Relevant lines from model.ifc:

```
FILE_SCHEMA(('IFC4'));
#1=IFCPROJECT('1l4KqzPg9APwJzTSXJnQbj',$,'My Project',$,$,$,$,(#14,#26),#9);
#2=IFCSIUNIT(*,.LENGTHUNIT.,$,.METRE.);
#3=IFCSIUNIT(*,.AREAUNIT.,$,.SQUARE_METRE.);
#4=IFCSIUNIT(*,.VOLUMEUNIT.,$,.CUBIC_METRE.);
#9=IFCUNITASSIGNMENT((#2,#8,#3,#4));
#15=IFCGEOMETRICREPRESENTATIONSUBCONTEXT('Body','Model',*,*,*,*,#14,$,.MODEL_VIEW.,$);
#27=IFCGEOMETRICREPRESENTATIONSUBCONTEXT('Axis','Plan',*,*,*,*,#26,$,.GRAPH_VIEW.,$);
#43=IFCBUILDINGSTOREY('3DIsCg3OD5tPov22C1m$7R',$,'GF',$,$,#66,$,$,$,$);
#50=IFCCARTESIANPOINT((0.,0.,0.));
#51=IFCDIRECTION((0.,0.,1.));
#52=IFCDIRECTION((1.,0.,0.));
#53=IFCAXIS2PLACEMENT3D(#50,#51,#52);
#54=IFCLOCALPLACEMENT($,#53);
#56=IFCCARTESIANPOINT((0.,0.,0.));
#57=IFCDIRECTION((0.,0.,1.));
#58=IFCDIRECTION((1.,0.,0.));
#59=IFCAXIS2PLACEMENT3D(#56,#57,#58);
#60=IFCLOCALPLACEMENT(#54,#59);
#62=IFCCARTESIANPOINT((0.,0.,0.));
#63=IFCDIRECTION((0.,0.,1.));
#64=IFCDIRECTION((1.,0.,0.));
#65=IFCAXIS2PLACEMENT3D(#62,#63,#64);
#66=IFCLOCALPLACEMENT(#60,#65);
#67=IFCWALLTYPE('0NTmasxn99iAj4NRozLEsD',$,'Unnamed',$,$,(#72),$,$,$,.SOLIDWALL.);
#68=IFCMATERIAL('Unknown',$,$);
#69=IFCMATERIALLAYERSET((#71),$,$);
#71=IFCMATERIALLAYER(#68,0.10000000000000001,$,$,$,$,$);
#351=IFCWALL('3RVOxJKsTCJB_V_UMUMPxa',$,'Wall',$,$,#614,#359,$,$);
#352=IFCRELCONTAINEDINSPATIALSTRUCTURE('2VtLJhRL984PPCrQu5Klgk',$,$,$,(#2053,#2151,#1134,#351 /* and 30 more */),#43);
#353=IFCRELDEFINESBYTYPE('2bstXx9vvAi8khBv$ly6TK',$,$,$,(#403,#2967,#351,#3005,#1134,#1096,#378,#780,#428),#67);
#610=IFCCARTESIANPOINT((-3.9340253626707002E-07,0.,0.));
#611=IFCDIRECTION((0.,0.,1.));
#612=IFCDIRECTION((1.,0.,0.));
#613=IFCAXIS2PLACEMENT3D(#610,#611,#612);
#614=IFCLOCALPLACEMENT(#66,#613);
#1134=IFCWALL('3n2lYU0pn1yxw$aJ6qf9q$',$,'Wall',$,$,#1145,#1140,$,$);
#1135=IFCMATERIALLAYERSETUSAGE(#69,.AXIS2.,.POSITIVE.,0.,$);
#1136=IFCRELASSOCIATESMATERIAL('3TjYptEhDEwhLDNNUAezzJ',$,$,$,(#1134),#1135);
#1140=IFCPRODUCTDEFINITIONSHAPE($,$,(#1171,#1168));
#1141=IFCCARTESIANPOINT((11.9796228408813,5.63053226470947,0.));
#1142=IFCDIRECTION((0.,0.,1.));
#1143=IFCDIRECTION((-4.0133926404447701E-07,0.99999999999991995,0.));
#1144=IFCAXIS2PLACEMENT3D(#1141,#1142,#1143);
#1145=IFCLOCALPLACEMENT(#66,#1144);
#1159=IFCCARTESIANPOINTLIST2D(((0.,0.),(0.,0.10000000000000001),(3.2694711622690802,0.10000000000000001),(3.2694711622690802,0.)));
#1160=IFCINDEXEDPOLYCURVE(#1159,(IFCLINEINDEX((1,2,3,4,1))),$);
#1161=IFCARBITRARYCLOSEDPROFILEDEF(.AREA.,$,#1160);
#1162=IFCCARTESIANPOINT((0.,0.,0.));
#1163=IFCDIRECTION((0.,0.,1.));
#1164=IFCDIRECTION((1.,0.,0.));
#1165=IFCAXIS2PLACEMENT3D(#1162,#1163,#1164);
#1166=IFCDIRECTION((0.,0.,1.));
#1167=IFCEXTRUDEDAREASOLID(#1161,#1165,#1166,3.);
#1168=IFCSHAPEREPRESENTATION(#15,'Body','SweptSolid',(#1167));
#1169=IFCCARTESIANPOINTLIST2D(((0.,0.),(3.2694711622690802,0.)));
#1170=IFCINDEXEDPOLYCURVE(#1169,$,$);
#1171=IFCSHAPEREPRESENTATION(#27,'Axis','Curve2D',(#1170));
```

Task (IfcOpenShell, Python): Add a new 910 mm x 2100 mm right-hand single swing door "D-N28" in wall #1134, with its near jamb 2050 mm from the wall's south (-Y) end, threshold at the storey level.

```python
import numpy as np
import ifcopenshell
import ifcopenshell.api.feature
import ifcopenshell.api.geometry
import ifcopenshell.api.root
import ifcopenshell.api.spatial
import ifcopenshell.geom
import ifcopenshell.util.element
import ifcopenshell.util.placement
import ifcopenshell.util.representation
import ifcopenshell.util.shape
import ifcopenshell.util.unit

model = ifcopenshell.open("model.ifc")
unit_scale = ifcopenshell.util.unit.calculate_unit_scale(model)
settings = ifcopenshell.geom.settings()


def volume(element):
    """Net volume in cubic metres, openings subtracted."""
    shape = ifcopenshell.geom.create_shape(settings, element)
    return ifcopenshell.util.shape.get_volume(shape.geometry)


wall = model.by_guid("3n2lYU0pn1yxw$aJ6qf9q$")
storey = ifcopenshell.util.element.get_container(wall, ifc_class="IfcBuildingStorey")
context = ifcopenshell.util.representation.get_context(model, "Model", "Body", "MODEL_VIEW")
before = volume(wall)

width, height, from_end, sill = 0.91, 2.1, 2.05, 0.0  # metres

# The wall runs along its own X axis, and the end named is its -X end.
wall_shape = ifcopenshell.geom.create_shape(settings, wall)
x, y, z = ifcopenshell.util.shape.get_vertices(wall_shape.geometry).T
start = x.min() + from_end
face, thickness = float(y.min()), float(y.max() - y.min())
wall_matrix = ifcopenshell.util.placement.get_local_placement(wall.ObjectPlacement)
level = ifcopenshell.util.placement.get_local_placement(storey.ObjectPlacement)[2, 3]


def in_wall(x, y):
    """Placement at x, y metres in the wall's axes, at sill height."""
    matrix = wall_matrix.copy()
    matrix[:, 3] = wall_matrix @ np.array([x / unit_scale, y / unit_scale, 0.0, 1.0])
    matrix[2, 3] = level + sill / unit_scale
    return matrix


# Opening: a box that overshoots both wall faces by 50 mm.
opening = ifcopenshell.api.root.create_entity(model, ifc_class="IfcOpeningElement", predefined_type="OPENING")
box = ifcopenshell.api.geometry.add_wall_representation(
    model, context=context, length=width, height=height, thickness=thickness + 0.1
)
ifcopenshell.api.geometry.assign_representation(model, product=opening, representation=box)
ifcopenshell.api.geometry.edit_object_placement(model, product=opening, matrix=in_wall(start, face - 0.05), is_si=False)
ifcopenshell.api.feature.add_feature(model, feature=opening, element=wall)

door = ifcopenshell.api.root.create_entity(model, ifc_class="IfcDoor", name="D-N28", predefined_type="DOOR")
door.OverallWidth, door.OverallHeight = width / unit_scale, height / unit_scale
door.OperationType = "SINGLE_SWING_RIGHT"
body = ifcopenshell.api.geometry.add_door_representation(
    model,
    context=context,
    overall_width=door.OverallWidth,
    overall_height=door.OverallHeight,
    operation_type="SINGLE_SWING_RIGHT",
    lining_properties={"LiningDepth": thickness / unit_scale, "ThresholdDepth": thickness / unit_scale},
)
ifcopenshell.api.geometry.assign_representation(model, product=door, representation=body)
ifcopenshell.api.spatial.assign_container(model, products=[door], relating_structure=storey)
ifcopenshell.api.feature.add_filling(model, opening=opening, element=door)

# The lining spans the wall, so the door starts at the wall face.
ifcopenshell.api.geometry.edit_object_placement(model, product=door, matrix=in_wall(start, face), is_si=False)

after = volume(wall)

print(f"wall volume {before:.3f} -> {after:.3f} m3")

model.write("model_updated.ifc")
```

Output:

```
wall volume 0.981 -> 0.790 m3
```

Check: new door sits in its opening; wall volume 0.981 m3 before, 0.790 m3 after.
